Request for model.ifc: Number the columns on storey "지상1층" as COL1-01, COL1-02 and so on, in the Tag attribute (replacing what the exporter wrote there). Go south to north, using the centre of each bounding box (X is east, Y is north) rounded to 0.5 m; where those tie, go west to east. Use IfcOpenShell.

First a look at what the model holds.

```python
import ifcopenshell
import ifcopenshell.util.element
import ifcopenshell.util.placement

model = ifcopenshell.open("model.ifc")
print(model.schema)
storey = next(s for s in model.by_type("IfcBuildingStorey") if s.Name == "지상1층")
columns = [e for e in ifcopenshell.util.element.get_decomposition(storey) if e.is_a("IfcColumn")]
for e in sorted(columns, key=lambda e: e.id()):
    origin = ifcopenshell.util.placement.get_local_placement(e.ObjectPlacement)[:3, 3]
    print(e.id(), e.Tag, e.Name, origin.round(2) + 0.0, sep=" | ")
```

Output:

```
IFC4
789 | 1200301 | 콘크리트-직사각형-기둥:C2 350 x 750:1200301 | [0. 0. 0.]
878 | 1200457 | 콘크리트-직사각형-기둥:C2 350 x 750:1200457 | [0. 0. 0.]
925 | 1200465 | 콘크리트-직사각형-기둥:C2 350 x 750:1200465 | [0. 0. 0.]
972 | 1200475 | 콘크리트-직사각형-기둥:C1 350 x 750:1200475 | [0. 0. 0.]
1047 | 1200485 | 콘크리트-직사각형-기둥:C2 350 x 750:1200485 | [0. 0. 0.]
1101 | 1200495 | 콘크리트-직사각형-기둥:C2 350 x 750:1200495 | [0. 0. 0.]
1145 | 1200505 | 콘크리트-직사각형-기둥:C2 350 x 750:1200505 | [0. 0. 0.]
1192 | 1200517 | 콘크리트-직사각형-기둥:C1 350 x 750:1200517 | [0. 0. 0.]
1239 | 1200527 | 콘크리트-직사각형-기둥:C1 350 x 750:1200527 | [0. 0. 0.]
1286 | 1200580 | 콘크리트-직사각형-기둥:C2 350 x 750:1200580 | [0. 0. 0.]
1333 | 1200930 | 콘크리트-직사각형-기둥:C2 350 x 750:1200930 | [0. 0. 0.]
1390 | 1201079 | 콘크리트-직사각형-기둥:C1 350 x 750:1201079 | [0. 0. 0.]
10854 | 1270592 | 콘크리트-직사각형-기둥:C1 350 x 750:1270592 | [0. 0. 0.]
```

```python
import ifcopenshell
import ifcopenshell.geom
import ifcopenshell.util.element
import ifcopenshell.util.shape

model = ifcopenshell.open("model.ifc")
settings = ifcopenshell.geom.settings()
settings.set("use-world-coords", True)


def centre(element):
    shape = ifcopenshell.geom.create_shape(settings, element)
    return ifcopenshell.util.shape.get_bbox_centroid(shape.geometry)


storey = next(s for s in model.by_type("IfcBuildingStorey") if s.Name == "지상1층")
columns = [e for e in ifcopenshell.util.element.get_decomposition(storey) if e.is_a("IfcColumn")]

# Insertion points can sit at a corner or the storey origin, so sort by the geometry (in metres).
centres = {e: centre(e) for e in columns}
columns.sort(key=lambda e: (round(centres[e][1] / 0.5), centres[e][0]))

for i, e in enumerate(columns, start=1):
    number = f"COL1-{i:02d}"
    e.Tag = number
    print(e.id(), number)

model.write("model-out.ifc")
```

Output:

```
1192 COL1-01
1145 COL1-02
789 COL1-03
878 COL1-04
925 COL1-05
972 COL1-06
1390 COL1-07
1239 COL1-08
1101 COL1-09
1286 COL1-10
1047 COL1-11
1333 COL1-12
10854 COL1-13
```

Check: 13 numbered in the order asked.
